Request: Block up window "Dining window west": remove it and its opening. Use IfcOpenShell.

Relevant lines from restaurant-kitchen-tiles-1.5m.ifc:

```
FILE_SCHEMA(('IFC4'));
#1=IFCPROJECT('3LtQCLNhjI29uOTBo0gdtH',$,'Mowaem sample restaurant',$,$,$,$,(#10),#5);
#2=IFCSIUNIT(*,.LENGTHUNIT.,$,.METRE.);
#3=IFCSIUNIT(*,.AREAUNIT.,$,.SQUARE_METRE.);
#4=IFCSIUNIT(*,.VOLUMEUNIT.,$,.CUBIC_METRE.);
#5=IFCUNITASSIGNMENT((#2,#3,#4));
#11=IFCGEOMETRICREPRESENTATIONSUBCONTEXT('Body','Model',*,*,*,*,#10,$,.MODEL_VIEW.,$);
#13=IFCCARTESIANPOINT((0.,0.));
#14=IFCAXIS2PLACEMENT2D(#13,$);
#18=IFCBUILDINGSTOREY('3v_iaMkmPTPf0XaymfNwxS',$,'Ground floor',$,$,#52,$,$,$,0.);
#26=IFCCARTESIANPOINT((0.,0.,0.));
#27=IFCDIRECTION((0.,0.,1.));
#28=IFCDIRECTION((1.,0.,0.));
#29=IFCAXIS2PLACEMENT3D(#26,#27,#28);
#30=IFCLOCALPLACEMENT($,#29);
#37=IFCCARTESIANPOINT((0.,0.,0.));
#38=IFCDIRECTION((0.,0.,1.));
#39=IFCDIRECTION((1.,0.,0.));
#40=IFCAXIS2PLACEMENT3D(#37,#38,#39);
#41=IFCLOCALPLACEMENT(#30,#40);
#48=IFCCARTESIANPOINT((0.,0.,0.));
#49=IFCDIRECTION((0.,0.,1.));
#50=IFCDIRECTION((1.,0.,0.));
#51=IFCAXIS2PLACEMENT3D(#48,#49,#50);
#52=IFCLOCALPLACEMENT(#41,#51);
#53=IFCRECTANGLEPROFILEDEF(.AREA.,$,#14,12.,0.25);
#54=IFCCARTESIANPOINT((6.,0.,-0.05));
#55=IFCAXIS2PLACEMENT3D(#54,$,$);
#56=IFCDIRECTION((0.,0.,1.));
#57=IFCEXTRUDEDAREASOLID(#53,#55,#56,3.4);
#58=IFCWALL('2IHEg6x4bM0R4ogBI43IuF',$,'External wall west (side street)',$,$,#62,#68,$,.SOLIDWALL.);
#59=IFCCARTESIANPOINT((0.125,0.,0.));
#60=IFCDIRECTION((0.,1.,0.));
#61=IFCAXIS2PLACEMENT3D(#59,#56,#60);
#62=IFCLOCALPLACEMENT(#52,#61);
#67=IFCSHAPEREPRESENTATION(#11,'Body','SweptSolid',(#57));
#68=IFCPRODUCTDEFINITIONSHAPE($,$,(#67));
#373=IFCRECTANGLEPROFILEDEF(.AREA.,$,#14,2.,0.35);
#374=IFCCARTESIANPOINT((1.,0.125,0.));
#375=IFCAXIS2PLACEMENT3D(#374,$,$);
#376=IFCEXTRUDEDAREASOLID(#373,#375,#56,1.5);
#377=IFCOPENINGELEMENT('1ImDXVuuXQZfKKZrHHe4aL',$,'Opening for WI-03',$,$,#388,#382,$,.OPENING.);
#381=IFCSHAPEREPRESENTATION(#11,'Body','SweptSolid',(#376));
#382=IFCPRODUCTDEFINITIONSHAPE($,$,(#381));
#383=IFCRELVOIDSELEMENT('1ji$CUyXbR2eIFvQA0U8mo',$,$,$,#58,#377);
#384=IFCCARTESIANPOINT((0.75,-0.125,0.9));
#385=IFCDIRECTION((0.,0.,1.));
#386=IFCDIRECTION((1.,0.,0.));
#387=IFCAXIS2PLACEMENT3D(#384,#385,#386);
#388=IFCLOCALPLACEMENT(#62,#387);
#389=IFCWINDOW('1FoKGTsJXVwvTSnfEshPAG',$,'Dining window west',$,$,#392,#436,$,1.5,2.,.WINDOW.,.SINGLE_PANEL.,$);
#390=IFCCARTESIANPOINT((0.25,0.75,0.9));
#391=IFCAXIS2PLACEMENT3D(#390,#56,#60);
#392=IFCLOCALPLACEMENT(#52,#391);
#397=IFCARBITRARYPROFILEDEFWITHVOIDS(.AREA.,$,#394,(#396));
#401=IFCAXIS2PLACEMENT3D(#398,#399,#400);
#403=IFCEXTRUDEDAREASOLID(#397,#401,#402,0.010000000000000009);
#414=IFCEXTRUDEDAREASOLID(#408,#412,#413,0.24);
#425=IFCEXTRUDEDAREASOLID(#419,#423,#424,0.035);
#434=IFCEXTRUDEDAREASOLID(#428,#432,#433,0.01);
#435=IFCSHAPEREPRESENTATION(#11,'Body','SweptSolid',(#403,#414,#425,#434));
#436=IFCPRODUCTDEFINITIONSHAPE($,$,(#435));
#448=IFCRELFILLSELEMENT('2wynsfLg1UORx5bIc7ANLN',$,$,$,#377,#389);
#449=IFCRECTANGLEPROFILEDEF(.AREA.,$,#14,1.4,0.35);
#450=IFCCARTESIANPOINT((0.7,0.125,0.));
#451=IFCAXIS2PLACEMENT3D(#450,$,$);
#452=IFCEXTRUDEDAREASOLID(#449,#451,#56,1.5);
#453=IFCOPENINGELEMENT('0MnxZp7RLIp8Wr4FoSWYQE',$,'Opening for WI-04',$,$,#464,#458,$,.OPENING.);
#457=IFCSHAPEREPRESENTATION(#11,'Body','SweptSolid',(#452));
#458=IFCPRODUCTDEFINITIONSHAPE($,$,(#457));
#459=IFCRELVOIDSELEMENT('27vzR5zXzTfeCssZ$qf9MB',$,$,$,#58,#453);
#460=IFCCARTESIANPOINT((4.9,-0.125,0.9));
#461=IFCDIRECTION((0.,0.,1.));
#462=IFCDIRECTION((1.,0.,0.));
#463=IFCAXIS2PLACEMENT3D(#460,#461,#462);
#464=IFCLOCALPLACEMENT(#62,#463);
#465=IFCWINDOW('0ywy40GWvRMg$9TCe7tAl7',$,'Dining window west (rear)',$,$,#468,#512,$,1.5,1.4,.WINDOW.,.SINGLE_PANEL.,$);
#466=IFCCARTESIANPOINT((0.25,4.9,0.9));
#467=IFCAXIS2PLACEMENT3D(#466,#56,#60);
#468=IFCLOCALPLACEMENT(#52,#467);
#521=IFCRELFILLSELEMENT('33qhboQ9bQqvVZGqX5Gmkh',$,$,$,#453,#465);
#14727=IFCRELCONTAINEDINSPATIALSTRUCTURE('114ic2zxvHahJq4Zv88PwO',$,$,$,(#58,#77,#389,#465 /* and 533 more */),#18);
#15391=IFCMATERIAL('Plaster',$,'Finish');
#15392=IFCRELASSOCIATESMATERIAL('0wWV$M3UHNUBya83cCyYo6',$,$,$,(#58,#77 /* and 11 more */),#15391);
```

```python
import ifcopenshell
import ifcopenshell.api.feature
import ifcopenshell.api.root
import ifcopenshell.geom
import ifcopenshell.util.shape

model = ifcopenshell.open("restaurant-kitchen-tiles-1.5m.ifc")
settings = ifcopenshell.geom.settings()


def volume(element):
    """Net volume in cubic metres, openings subtracted."""
    shape = ifcopenshell.geom.create_shape(settings, element)
    return ifcopenshell.util.shape.get_volume(shape.geometry)


window = model.by_guid("1FoKGTsJXVwvTSnfEshPAG")
opening = window.FillsVoids[0].RelatingOpeningElement
wall = opening.VoidsElements[0].RelatingBuildingElement
before = volume(wall)

ifcopenshell.api.root.remove_product(model, product=window)
ifcopenshell.api.feature.remove_feature(model, feature=opening)

after = volume(wall)

print(f"wall volume {before:.3f} -> {after:.3f} m3")

model.write("restaurant-kitchen-tiles-1.5m-out.ifc")
```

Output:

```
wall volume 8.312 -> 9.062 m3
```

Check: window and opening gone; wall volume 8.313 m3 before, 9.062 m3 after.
